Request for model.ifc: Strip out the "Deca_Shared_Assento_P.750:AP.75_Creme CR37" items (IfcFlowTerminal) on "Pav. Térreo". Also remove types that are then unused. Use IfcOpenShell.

First a look at what the model holds.

```python
import ifcopenshell
import ifcopenshell.util.element

model = ifcopenshell.open("model.ifc")
print(model.schema)
storey = next(s for s in model.by_type("IfcBuildingStorey") if s.Name == "Pav. Térreo")
terminals = [e for e in ifcopenshell.util.element.get_decomposition(storey) if e.is_a("IfcFlowTerminal")]
seen = {}
for e in terminals:
    element_type = ifcopenshell.util.element.get_type(e)
    name = element_type.Name if element_type not in (None, e) else None
    seen[name] = seen.get(name, 0) + 1
for name, count in sorted(seen.items(), key=str):
    print(count, "x", name)
```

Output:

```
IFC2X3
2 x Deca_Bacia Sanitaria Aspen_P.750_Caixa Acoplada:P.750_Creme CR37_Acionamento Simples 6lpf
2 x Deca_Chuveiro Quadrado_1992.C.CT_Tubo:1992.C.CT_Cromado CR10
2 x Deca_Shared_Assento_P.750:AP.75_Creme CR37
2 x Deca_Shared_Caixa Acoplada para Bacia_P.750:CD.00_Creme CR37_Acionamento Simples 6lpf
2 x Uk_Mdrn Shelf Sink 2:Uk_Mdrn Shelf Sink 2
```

```python
import ifcopenshell
import ifcopenshell.api.root
import ifcopenshell.util.element

model = ifcopenshell.open("model.ifc")

storey = next(s for s in model.by_type("IfcBuildingStorey") if s.Name == "Pav. Térreo")
terminals = [e for e in ifcopenshell.util.element.get_decomposition(storey) if e.is_a("IfcFlowTerminal")]
targets = [e for e in terminals if (t := ifcopenshell.util.element.get_type(e)) not in (None, e) and t.Name == "Deca_Shared_Assento_P.750:AP.75_Creme CR37"]
types = {ifcopenshell.util.element.get_type(e) for e in targets} - {None, *targets}

for e in targets:
    ifcopenshell.api.root.remove_product(model, product=e)
print(len(targets), "removed")

unused = [t for t in types if not ifcopenshell.util.element.get_types(t)]
for t in unused:
    ifcopenshell.api.root.remove_product(model, product=t)
print(len(unused), "unused types removed")

model.write("model_rev.ifc")
```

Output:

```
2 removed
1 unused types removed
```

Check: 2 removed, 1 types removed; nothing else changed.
